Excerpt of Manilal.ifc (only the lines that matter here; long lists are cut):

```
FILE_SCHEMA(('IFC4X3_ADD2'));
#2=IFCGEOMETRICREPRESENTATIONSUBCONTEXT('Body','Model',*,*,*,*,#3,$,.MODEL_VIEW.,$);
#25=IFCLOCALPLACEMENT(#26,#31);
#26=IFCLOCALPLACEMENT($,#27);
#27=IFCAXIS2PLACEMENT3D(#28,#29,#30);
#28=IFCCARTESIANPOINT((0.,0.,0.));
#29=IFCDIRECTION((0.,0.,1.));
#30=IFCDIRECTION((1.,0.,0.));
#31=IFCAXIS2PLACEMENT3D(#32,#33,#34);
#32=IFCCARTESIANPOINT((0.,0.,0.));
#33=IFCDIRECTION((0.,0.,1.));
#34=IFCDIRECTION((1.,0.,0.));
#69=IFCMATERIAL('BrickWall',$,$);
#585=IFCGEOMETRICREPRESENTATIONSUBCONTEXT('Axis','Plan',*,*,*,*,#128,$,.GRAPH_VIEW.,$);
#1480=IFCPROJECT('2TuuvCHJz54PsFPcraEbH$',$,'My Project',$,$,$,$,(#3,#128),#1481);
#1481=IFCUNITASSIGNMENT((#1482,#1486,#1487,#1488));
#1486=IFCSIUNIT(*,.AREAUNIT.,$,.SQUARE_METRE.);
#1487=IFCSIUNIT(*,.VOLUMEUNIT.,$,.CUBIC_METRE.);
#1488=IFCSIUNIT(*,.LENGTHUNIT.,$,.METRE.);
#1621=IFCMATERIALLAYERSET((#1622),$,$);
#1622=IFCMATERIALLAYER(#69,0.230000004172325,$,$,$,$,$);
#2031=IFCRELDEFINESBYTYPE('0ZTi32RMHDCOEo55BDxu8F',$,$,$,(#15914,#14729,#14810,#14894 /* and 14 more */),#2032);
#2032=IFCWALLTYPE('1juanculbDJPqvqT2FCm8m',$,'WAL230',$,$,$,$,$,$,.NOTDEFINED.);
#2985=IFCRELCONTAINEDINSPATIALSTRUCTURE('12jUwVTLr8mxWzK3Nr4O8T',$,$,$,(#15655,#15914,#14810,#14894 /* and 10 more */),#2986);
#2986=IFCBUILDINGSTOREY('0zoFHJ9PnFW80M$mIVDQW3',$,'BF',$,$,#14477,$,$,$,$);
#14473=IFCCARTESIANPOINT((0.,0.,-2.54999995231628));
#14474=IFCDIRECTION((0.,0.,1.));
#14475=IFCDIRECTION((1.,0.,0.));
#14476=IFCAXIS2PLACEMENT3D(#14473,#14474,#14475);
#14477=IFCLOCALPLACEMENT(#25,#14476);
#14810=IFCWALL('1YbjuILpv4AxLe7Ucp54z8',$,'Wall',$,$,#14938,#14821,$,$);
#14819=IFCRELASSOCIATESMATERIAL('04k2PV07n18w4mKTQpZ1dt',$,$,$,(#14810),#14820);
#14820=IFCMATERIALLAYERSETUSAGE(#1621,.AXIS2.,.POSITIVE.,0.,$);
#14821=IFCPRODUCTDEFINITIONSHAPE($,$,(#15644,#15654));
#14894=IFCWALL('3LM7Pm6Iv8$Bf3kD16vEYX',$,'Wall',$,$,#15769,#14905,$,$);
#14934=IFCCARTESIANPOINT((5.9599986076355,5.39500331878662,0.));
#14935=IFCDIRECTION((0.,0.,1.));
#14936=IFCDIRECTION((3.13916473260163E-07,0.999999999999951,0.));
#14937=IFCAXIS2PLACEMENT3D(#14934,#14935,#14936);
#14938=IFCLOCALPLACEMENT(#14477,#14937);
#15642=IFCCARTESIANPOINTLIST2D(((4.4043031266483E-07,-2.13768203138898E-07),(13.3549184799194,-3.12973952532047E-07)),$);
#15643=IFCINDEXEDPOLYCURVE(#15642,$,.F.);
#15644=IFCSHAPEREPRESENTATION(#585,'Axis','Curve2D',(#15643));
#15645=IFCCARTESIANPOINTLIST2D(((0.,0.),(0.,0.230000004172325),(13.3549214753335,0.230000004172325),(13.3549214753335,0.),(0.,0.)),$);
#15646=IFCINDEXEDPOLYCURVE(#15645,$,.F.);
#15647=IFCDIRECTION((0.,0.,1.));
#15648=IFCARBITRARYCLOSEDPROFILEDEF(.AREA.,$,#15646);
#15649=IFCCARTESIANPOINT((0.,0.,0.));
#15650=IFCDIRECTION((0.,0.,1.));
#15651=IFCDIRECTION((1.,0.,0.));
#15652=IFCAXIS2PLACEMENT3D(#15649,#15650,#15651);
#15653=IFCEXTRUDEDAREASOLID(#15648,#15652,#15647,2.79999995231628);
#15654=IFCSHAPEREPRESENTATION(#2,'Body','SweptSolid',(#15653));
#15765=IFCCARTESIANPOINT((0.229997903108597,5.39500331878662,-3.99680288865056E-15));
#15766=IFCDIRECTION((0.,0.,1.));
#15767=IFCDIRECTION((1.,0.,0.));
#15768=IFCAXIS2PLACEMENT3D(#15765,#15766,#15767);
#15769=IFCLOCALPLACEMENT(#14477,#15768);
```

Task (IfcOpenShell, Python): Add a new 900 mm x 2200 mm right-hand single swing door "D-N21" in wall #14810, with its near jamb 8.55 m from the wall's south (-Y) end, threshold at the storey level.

```python
import numpy as np
import ifcopenshell
import ifcopenshell.api.feature
import ifcopenshell.api.geometry
import ifcopenshell.api.root
import ifcopenshell.api.spatial
import ifcopenshell.geom
import ifcopenshell.util.element
import ifcopenshell.util.placement
import ifcopenshell.util.representation
import ifcopenshell.util.shape
import ifcopenshell.util.unit

model = ifcopenshell.open("Manilal.ifc")
unit_scale = ifcopenshell.util.unit.calculate_unit_scale(model)
settings = ifcopenshell.geom.settings()


def volume(element):
    """Net volume in cubic metres, openings subtracted."""
    shape = ifcopenshell.geom.create_shape(settings, element)
    return ifcopenshell.util.shape.get_volume(shape.geometry)


wall = model.by_id(14810)
storey = ifcopenshell.util.element.get_container(wall, ifc_class="IfcBuildingStorey")
context = ifcopenshell.util.representation.get_context(model, "Model", "Body", "MODEL_VIEW")
before = volume(wall)

width, height, from_end, sill = 0.9, 2.2, 8.55, 0.0  # metres

# The wall runs along its own X axis, and the end named is its -X end.
wall_shape = ifcopenshell.geom.create_shape(settings, wall)
x, y, z = ifcopenshell.util.shape.get_vertices(wall_shape.geometry).T
start = x.min() + from_end
face, thickness = float(y.min()), float(y.max() - y.min())
wall_matrix = ifcopenshell.util.placement.get_local_placement(wall.ObjectPlacement)
level = ifcopenshell.util.placement.get_local_placement(storey.ObjectPlacement)[2, 3]


def in_wall(x, y):
    """Placement at x, y metres in the wall's axes, at sill height."""
    matrix = wall_matrix.copy()
    matrix[:, 3] = wall_matrix @ np.array([x / unit_scale, y / unit_scale, 0.0, 1.0])
    matrix[2, 3] = level + sill / unit_scale
    return matrix


# Opening: a box that overshoots both wall faces by 50 mm.
opening = ifcopenshell.api.root.create_entity(model, ifc_class="IfcOpeningElement", predefined_type="OPENING")
box = ifcopenshell.api.geometry.add_wall_representation(
    model, context=context, length=width, height=height, thickness=thickness + 0.1
)
ifcopenshell.api.geometry.assign_representation(model, product=opening, representation=box)
ifcopenshell.api.geometry.edit_object_placement(model, product=opening, matrix=in_wall(start, face - 0.05), is_si=False)
ifcopenshell.api.feature.add_feature(model, feature=opening, element=wall)

door = ifcopenshell.api.root.create_entity(model, ifc_class="IfcDoor", name="D-N21", predefined_type="DOOR")
door.OverallWidth, door.OverallHeight = width / unit_scale, height / unit_scale
door.OperationType = "SINGLE_SWING_RIGHT"
body = ifcopenshell.api.geometry.add_door_representation(
    model,
    context=context,
    overall_width=door.OverallWidth,
    overall_height=door.OverallHeight,
    operation_type="SINGLE_SWING_RIGHT",
    lining_properties={"LiningDepth": thickness / unit_scale, "ThresholdDepth": thickness / unit_scale},
)
ifcopenshell.api.geometry.assign_representation(model, product=door, representation=body)
ifcopenshell.api.spatial.assign_container(model, products=[door], relating_structure=storey)
ifcopenshell.api.feature.add_filling(model, opening=opening, element=door)

# The lining spans the wall, so the door starts at the wall face.
ifcopenshell.api.geometry.edit_object_placement(model, product=door, matrix=in_wall(start, face), is_si=False)

after = volume(wall)

print(f"wall volume {before:.3f} -> {after:.3f} m3")

model.write("Manilal_v2.ifc")
```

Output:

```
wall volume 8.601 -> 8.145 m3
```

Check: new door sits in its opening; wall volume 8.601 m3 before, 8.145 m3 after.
